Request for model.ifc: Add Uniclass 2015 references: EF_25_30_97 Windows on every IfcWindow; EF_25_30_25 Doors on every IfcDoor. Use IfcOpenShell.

First a look at what the model holds.

```python
import ifcopenshell

model = ifcopenshell.open("model.ifc")
print(model.schema)
print("classifications:", [c.Name for c in model.by_type("IfcClassification")])
for ifc_class in ("IfcDoor", "IfcRoof", "IfcStair", "IfcWall", "IfcWindow"):
    print(ifc_class, len(model.by_type(ifc_class)))
```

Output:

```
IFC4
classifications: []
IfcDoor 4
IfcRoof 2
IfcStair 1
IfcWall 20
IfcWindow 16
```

```python
import ifcopenshell
import ifcopenshell.api.classification

model = ifcopenshell.open("model.ifc")

system = ifcopenshell.api.classification.add_classification(model, classification="Uniclass 2015")

codes = {
    "IfcWindow": ("EF_25_30_97", "Windows"),
    "IfcDoor": ("EF_25_30_25", "Doors"),
}
for ifc_class, (code, name) in codes.items():
    products = model.by_type(ifc_class)
    ifcopenshell.api.classification.add_reference(
        model, products=products, classification=system, identification=code, name=name
    )
    print(code, len(products))

model.write("model_updated.ifc")
```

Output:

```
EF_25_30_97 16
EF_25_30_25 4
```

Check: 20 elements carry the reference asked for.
